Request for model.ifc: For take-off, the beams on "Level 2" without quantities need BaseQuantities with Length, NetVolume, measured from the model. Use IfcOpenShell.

First a look at what the model holds.

```python
import ifcopenshell
import ifcopenshell.util.element
import ifcopenshell.util.unit

model = ifcopenshell.open("model.ifc")
print(model.schema)
for unit_type in ("LENGTHUNIT", "AREAUNIT", "VOLUMEUNIT"):
    print(unit_type, ifcopenshell.util.unit.calculate_unit_scale(model, unit_type))
storey = next(s for s in model.by_type("IfcBuildingStorey") if s.Name == "Level 2")
beams = [e for e in ifcopenshell.util.element.get_decomposition(storey) if e.is_a("IfcBeam")]
for e in sorted(beams, key=lambda e: e.id()):
    print(e.id(), e.is_a(), e.Name, list(ifcopenshell.util.element.get_psets(e, qtos_only=True)), sep=" | ")
```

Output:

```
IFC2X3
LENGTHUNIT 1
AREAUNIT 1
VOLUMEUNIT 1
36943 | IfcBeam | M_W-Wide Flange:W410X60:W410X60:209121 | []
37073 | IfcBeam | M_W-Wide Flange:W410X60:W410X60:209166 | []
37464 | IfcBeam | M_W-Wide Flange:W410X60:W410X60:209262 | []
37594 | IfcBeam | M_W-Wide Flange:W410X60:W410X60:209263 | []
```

```python
import ifcopenshell
import ifcopenshell.api.pset
import ifcopenshell.geom
import ifcopenshell.util.element
import ifcopenshell.util.shape
import ifcopenshell.util.unit

model = ifcopenshell.open("model.ifc")
unit_scale = ifcopenshell.util.unit.calculate_unit_scale(model)
volume_scale = ifcopenshell.util.unit.calculate_unit_scale(model, "VOLUMEUNIT")
settings = ifcopenshell.geom.settings()

storey = next(s for s in model.by_type("IfcBuildingStorey") if s.Name == "Level 2")
beams = [e for e in ifcopenshell.util.element.get_decomposition(storey) if e.is_a("IfcBeam")]

for e in sorted(beams, key=lambda e: e.id()):
    if ifcopenshell.util.element.get_psets(e, qtos_only=True, should_inherit=False):
        continue
    # Geometry comes back in metres, in the element's own axes.
    shape = ifcopenshell.geom.create_shape(settings, e)
    values = {
        "Length": ifcopenshell.util.shape.get_max_xyz(shape.geometry) / unit_scale,
        "NetVolume": ifcopenshell.util.shape.get_volume(shape.geometry) / volume_scale,
    }
    qto = ifcopenshell.api.pset.add_qto(model, product=e, name="BaseQuantities")
    ifcopenshell.api.pset.edit_qto(model, qto=qto, properties=values)
    print(e.id(), {k: round(v, 3) for k, v in values.items()})

model.write("model-out.ifc")
```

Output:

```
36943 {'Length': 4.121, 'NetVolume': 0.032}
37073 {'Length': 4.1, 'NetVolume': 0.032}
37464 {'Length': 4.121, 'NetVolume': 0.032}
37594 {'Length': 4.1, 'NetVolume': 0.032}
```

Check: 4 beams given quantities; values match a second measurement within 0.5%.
